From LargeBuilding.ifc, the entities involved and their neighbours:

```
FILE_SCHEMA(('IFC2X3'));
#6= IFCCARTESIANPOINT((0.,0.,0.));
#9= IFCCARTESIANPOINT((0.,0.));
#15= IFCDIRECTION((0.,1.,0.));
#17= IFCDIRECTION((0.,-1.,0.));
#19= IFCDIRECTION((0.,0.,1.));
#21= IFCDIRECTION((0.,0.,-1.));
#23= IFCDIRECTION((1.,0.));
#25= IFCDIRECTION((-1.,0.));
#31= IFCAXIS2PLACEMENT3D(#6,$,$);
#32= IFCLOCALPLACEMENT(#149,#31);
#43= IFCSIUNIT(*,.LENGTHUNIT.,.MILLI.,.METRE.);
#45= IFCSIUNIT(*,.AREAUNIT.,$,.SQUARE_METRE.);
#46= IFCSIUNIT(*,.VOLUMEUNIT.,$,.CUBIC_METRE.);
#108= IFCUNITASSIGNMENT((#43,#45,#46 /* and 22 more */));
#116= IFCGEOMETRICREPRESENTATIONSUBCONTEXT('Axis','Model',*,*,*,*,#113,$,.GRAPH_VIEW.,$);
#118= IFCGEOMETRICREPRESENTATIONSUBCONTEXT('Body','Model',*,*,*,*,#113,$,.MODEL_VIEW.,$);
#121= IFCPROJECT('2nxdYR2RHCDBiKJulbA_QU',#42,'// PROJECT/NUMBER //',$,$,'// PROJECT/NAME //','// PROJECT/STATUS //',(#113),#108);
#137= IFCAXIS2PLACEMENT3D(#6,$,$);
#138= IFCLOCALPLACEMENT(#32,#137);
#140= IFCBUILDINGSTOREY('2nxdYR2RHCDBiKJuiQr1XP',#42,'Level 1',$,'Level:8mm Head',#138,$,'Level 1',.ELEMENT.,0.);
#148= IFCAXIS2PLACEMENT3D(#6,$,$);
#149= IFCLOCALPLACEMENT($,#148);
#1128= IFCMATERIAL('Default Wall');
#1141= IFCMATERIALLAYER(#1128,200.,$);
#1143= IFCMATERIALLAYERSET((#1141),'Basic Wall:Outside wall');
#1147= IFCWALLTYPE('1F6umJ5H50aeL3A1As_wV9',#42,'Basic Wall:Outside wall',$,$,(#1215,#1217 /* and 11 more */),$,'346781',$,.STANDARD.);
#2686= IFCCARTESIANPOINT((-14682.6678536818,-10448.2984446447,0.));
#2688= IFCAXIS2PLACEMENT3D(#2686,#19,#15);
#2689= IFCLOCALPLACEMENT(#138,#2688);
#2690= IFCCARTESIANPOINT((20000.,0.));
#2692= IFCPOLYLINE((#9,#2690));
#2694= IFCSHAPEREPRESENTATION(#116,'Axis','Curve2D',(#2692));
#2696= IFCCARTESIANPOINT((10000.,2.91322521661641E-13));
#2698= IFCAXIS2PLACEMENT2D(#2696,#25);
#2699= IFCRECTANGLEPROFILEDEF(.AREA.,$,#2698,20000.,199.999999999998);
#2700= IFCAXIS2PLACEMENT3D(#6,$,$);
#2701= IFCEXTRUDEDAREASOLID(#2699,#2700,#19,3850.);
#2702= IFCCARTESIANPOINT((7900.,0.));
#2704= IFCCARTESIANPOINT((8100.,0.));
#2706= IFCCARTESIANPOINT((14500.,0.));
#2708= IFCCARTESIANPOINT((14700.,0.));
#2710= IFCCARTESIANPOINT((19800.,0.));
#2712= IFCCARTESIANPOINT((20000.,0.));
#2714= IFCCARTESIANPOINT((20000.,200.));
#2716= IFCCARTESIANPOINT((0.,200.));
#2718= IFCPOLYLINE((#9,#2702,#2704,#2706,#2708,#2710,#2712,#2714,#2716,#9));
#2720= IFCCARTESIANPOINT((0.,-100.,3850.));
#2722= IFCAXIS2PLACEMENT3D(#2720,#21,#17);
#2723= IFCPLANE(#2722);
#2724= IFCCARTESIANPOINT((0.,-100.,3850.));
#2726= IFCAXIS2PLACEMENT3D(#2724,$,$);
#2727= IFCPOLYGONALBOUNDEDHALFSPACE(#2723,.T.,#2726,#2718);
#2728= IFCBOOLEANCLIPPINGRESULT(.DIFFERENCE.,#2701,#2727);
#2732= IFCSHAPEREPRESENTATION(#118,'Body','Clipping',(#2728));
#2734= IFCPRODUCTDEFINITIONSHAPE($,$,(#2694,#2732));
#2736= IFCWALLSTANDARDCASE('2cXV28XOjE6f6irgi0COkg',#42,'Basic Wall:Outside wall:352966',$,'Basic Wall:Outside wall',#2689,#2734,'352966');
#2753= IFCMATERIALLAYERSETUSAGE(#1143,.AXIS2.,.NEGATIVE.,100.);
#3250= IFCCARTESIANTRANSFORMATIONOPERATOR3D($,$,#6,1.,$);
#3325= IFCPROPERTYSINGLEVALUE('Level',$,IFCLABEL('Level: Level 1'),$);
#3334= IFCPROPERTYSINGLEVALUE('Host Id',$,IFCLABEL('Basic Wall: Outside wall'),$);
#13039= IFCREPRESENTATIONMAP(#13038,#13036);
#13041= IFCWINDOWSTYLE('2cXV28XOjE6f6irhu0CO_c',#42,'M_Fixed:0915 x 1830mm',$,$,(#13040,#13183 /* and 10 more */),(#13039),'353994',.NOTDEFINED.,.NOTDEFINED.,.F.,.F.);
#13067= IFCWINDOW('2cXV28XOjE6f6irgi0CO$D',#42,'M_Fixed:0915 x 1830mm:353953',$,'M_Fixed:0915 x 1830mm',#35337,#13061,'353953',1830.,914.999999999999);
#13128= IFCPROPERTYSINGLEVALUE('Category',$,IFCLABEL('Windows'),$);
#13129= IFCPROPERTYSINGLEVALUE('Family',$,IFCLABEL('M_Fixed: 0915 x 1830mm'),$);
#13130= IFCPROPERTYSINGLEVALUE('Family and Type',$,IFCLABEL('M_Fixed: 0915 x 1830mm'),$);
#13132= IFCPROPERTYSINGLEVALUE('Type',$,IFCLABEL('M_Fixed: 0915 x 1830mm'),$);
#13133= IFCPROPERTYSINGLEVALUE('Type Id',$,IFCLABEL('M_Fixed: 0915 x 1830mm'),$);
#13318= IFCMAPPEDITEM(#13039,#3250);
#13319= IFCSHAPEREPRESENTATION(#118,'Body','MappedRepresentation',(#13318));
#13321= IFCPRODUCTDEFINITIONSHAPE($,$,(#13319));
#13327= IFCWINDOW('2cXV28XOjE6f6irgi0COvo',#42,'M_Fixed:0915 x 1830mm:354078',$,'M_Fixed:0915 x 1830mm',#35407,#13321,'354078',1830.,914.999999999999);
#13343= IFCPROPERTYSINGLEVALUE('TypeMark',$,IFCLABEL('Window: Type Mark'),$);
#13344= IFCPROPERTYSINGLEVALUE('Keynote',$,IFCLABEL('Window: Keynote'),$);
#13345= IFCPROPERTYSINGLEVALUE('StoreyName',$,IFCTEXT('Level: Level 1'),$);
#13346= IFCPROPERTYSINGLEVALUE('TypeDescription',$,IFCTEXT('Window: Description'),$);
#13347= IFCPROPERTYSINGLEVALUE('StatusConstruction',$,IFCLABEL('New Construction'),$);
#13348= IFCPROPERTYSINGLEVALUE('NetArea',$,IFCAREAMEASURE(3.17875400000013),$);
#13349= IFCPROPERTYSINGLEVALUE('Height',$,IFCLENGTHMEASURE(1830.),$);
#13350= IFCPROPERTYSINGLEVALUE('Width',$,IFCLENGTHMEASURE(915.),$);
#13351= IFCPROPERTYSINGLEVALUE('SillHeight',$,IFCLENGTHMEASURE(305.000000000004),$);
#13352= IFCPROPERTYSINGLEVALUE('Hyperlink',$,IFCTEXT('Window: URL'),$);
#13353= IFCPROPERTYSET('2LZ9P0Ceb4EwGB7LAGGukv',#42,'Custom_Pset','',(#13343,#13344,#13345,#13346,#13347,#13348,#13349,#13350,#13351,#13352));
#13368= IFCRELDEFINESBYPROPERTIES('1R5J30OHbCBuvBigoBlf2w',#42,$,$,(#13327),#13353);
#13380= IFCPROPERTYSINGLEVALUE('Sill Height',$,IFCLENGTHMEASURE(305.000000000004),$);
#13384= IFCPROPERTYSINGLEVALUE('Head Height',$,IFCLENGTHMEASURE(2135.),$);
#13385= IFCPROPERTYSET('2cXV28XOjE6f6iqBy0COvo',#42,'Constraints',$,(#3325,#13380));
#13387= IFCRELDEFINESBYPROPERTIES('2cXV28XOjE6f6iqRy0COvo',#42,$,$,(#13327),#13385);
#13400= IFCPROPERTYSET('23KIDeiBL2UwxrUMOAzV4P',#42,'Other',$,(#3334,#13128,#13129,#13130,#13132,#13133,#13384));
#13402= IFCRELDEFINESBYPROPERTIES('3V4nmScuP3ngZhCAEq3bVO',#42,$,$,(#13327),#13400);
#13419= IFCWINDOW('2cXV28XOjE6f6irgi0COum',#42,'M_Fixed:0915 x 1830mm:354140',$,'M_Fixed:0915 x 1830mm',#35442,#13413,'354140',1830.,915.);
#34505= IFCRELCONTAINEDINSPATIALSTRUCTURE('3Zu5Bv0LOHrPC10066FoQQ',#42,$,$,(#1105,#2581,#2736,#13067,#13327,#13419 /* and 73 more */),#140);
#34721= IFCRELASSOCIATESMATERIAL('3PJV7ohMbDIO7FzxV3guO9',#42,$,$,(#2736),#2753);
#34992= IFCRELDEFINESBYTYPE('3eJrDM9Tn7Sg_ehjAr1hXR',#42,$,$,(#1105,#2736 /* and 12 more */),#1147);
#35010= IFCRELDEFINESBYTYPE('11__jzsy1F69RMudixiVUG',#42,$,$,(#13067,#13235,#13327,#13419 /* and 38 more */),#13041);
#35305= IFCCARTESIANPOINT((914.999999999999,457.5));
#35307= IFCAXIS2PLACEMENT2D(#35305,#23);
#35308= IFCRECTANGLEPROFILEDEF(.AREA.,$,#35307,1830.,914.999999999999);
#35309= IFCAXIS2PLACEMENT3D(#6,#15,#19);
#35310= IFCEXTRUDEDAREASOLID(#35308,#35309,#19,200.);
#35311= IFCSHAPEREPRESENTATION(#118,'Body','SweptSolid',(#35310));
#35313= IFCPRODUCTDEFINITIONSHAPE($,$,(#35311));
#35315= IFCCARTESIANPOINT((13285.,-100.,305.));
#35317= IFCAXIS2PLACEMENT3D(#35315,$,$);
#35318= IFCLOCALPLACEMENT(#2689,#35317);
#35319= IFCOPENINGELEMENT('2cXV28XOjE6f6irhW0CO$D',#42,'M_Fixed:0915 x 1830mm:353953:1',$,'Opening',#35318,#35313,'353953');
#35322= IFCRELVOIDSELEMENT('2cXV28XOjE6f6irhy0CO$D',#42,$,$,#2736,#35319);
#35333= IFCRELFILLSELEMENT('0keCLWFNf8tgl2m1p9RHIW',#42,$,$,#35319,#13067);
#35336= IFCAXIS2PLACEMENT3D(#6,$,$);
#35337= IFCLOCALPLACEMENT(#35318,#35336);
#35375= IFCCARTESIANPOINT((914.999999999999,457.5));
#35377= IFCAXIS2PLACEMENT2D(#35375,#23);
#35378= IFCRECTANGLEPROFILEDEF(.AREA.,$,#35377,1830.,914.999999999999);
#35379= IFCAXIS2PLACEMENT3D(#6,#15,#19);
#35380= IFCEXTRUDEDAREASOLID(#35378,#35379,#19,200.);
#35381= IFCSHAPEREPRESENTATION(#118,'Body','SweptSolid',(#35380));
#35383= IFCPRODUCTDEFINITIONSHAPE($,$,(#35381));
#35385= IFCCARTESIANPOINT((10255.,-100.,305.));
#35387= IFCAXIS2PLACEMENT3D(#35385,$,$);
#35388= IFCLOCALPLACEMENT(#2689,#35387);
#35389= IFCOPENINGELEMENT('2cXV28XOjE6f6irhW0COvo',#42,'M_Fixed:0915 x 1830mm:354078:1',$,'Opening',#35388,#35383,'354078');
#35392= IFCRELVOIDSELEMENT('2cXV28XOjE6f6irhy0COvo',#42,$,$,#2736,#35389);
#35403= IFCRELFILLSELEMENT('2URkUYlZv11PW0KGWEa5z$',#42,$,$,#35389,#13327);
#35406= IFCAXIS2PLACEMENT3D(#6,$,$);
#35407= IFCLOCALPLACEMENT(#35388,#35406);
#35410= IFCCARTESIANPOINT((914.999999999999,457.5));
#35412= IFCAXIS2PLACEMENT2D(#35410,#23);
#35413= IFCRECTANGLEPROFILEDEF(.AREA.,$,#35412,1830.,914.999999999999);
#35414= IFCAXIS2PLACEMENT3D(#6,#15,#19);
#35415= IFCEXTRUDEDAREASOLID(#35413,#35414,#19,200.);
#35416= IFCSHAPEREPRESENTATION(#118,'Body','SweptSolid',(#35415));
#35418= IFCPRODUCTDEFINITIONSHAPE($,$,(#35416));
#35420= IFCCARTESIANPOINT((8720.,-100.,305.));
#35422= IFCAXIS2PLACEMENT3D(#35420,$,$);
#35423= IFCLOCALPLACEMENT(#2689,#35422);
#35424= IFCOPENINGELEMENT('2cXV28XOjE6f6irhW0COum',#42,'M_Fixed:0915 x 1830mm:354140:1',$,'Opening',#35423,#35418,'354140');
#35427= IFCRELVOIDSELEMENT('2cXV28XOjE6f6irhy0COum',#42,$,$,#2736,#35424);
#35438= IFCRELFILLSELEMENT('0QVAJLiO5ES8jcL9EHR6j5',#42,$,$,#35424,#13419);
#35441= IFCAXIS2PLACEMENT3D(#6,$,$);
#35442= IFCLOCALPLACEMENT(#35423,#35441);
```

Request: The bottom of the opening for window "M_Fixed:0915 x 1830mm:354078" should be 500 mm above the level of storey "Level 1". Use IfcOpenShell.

```python
import numpy as np
import ifcopenshell
import ifcopenshell.api.geometry
import ifcopenshell.api.pset
import ifcopenshell.geom
import ifcopenshell.util.element
import ifcopenshell.util.placement
import ifcopenshell.util.shape
import ifcopenshell.util.unit

model = ifcopenshell.open("LargeBuilding.ifc")
unit_scale = ifcopenshell.util.unit.calculate_unit_scale(model)

window = model.by_guid("2cXV28XOjE6f6irgi0COvo")
opening = window.FillsVoids[0].RelatingOpeningElement
storey = ifcopenshell.util.element.get_container(window, ifc_class="IfcBuildingStorey")
level = ifcopenshell.util.placement.get_local_placement(storey.ObjectPlacement)[2, 3]

# The opening's origin need not be at the sill, so measure its lowest point.
shape = ifcopenshell.geom.create_shape(ifcopenshell.geom.settings(), opening)
bottom = ifcopenshell.util.shape.get_shape_bottom_elevation(shape, shape.geometry) / unit_scale
dz = level + 0.5 / unit_scale - bottom

shift = np.array([0.0, 0.0, dz])
# The window is placed relative to its opening, so it follows when the opening moves.
matrix = ifcopenshell.util.placement.get_local_placement(opening.ObjectPlacement)
matrix[:3, 3] += shift
ifcopenshell.api.geometry.edit_object_placement(
    model, product=opening, matrix=matrix, is_si=False, should_transform_children=True
)

# Keep the stored heights in step.
pset = model.by_id(ifcopenshell.util.element.get_pset(window, "Custom_Pset", should_inherit=False)["id"])
ifcopenshell.api.pset.edit_pset(model, pset=pset, properties={
    "SillHeight": model.create_entity("IfcLengthMeasure", ifcopenshell.util.element.get_pset(window, "Constraints", "Sill Height") + dz),
})
pset = model.by_id(ifcopenshell.util.element.get_pset(window, "Constraints", should_inherit=False)["id"])
ifcopenshell.api.pset.edit_pset(model, pset=pset, properties={
    "Sill Height": model.create_entity("IfcLengthMeasure", ifcopenshell.util.element.get_pset(window, "Constraints", "Sill Height") + dz),
})
pset = model.by_id(ifcopenshell.util.element.get_pset(window, "Other", should_inherit=False)["id"])
ifcopenshell.api.pset.edit_pset(model, pset=pset, properties={
    "Head Height": model.create_entity("IfcLengthMeasure", ifcopenshell.util.element.get_pset(window, "Other", "Head Height") + dz),
})

print(f"moved by {dz * unit_scale:+.3f} m")

model.write("LargeBuilding_v2.ifc")
```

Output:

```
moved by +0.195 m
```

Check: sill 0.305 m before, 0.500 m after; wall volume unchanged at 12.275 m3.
